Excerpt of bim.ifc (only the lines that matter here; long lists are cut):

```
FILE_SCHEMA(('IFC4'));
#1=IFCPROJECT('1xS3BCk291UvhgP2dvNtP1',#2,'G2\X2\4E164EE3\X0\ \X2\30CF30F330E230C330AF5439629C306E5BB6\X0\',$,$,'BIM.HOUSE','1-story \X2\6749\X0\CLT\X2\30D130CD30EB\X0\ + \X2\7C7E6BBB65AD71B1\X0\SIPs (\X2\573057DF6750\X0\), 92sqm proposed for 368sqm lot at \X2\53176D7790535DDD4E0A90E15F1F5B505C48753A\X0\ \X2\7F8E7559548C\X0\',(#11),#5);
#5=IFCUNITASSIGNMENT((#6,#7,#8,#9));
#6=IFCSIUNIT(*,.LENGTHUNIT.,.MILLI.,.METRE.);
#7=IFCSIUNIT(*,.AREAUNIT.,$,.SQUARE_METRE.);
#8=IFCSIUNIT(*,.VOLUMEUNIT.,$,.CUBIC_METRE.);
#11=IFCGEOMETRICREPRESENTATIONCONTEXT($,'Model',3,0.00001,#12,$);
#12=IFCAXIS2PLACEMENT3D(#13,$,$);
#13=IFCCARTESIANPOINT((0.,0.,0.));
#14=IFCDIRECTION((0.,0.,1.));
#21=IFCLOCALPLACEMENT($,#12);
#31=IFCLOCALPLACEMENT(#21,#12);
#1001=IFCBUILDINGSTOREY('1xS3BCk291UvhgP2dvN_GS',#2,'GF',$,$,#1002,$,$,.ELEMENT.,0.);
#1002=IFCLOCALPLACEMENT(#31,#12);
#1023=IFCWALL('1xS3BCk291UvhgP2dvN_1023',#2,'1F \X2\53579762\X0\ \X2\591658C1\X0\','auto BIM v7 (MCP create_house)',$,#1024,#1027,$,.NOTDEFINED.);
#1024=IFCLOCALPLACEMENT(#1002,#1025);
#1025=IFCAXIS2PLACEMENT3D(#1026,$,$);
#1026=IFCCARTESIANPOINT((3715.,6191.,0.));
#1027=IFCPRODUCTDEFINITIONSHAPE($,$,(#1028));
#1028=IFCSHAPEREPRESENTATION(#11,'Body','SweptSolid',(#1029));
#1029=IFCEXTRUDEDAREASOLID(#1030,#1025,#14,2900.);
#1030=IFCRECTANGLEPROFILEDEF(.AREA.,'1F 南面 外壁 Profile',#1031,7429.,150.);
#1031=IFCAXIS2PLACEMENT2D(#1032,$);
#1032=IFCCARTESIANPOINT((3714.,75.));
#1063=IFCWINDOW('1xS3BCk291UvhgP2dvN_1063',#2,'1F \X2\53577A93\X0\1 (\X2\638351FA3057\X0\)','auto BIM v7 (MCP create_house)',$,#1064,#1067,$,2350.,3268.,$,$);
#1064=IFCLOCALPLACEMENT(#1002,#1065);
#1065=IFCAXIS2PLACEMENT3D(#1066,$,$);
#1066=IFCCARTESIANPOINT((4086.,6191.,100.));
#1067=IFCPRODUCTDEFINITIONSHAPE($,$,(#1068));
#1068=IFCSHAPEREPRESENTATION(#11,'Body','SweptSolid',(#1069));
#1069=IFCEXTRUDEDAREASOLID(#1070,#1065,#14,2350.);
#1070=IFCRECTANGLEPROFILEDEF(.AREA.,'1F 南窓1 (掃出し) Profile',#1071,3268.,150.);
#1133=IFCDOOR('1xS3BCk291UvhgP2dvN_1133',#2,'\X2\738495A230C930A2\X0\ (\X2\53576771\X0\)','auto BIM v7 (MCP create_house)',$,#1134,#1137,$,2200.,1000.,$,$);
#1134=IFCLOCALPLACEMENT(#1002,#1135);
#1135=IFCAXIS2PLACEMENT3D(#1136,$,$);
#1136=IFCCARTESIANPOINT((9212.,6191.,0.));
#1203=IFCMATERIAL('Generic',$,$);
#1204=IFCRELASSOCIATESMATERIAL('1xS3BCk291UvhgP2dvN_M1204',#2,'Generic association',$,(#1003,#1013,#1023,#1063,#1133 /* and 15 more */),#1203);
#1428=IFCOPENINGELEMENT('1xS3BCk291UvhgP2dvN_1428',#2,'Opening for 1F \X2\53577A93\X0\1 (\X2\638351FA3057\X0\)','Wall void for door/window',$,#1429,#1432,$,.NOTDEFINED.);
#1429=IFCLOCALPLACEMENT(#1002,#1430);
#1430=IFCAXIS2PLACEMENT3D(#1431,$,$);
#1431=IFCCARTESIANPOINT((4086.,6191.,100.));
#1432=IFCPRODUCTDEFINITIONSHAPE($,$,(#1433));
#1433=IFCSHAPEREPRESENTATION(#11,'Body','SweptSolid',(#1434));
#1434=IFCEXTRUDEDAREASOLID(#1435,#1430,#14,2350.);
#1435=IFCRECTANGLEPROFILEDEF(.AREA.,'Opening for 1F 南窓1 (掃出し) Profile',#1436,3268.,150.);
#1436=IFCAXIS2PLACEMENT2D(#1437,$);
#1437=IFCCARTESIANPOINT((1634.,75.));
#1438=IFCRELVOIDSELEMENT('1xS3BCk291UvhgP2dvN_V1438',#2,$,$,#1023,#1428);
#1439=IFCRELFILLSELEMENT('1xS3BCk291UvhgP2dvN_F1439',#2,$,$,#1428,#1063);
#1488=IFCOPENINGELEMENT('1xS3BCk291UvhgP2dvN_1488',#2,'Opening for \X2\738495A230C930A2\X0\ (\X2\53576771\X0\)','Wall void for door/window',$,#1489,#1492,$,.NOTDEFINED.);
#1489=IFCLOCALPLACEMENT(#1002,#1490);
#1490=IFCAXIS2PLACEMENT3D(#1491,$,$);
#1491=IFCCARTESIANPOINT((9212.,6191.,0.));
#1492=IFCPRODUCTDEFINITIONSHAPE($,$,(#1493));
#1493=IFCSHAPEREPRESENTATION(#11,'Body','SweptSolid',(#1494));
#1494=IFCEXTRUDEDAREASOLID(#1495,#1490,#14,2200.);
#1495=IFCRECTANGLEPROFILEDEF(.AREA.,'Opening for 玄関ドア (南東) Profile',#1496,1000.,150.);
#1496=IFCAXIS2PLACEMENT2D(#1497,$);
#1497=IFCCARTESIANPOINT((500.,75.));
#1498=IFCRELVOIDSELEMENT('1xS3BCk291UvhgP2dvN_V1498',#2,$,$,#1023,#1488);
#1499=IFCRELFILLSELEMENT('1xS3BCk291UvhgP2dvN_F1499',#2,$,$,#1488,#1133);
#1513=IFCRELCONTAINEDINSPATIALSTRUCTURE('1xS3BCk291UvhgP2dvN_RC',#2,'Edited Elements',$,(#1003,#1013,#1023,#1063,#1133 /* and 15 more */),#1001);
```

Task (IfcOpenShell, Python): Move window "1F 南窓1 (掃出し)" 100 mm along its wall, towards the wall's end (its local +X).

```python
import ifcopenshell
import ifcopenshell.api.geometry
import ifcopenshell.util.placement
import ifcopenshell.util.unit

model = ifcopenshell.open("bim.ifc")
unit_scale = ifcopenshell.util.unit.calculate_unit_scale(model)

window = model.by_guid("1xS3BCk291UvhgP2dvN_1063")
opening = window.FillsVoids[0].RelatingOpeningElement
wall = opening.VoidsElements[0].RelatingBuildingElement

wall_matrix = ifcopenshell.util.placement.get_local_placement(wall.ObjectPlacement)
shift = wall_matrix[:3, 0] * 0.1 / unit_scale
before = ifcopenshell.util.placement.get_local_placement(window.ObjectPlacement)[:3, 3].copy()

# The window is not placed relative to its opening, so move both.
for product in (opening, window):
    matrix = ifcopenshell.util.placement.get_local_placement(product.ObjectPlacement)
    matrix[:3, 3] += shift
    ifcopenshell.api.geometry.edit_object_placement(model, product=product, matrix=matrix, is_si=False)

after = ifcopenshell.util.placement.get_local_placement(window.ObjectPlacement)[:3, 3]
print("window moved by", (after - before).round(3) + 0.0)

model.write("bim_v2.ifc")
```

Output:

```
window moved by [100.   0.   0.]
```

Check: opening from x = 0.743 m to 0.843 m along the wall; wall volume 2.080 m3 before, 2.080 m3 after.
